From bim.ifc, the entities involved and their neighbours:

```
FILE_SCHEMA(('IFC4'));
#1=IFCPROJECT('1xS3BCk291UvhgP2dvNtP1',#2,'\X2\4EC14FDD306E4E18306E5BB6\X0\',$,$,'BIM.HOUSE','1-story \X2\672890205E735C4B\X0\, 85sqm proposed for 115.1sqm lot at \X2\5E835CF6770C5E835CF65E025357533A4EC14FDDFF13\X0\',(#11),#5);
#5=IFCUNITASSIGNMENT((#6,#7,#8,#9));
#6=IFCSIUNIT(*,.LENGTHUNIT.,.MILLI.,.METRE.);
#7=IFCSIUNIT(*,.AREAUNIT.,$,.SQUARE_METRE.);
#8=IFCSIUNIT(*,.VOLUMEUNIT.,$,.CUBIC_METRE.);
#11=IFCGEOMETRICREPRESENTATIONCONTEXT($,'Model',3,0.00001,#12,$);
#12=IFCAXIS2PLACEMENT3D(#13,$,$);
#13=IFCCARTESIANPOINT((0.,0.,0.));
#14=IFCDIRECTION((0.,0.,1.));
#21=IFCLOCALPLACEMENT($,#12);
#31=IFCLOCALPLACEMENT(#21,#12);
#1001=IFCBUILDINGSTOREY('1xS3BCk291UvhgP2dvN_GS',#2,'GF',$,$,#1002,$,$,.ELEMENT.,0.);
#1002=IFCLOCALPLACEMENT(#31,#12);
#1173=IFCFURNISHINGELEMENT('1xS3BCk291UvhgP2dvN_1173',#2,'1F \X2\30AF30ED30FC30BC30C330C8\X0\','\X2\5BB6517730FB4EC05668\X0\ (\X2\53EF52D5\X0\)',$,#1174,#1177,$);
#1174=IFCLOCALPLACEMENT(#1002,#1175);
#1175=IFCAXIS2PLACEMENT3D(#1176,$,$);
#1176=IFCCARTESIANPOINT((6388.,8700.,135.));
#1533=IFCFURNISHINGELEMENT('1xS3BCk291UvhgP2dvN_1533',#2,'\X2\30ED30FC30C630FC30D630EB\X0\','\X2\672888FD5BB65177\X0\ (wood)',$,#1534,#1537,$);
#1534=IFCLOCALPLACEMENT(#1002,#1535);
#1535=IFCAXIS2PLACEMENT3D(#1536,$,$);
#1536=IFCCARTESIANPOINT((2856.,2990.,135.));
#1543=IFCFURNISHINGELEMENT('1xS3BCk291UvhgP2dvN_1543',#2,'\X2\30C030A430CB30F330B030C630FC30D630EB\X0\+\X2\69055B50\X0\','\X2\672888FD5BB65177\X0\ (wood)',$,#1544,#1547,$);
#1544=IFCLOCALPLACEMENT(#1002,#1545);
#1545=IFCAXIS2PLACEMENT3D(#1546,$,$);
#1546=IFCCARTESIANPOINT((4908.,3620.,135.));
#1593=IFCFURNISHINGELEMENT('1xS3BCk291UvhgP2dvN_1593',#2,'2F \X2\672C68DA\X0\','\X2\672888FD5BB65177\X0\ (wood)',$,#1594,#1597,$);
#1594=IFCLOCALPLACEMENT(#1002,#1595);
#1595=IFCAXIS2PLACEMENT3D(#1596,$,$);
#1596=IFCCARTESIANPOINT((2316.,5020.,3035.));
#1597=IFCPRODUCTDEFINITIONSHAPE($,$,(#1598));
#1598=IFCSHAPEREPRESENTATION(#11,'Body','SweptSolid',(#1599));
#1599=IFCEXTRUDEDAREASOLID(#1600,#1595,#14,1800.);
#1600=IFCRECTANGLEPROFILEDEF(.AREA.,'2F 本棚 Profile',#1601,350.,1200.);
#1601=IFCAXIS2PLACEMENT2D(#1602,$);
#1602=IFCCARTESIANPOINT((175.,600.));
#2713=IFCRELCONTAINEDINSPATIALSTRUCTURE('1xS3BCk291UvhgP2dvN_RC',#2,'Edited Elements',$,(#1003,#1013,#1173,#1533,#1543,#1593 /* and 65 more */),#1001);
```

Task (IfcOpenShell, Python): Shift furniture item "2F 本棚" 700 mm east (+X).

```python
import ifcopenshell
import ifcopenshell.api.geometry
import ifcopenshell.util.placement
import ifcopenshell.util.unit

model = ifcopenshell.open("bim.ifc")
unit_scale = ifcopenshell.util.unit.calculate_unit_scale(model)

item = model.by_guid("1xS3BCk291UvhgP2dvN_1593")
matrix = ifcopenshell.util.placement.get_local_placement(item.ObjectPlacement)
matrix[0, 3] += 0.7 / unit_scale
ifcopenshell.api.geometry.edit_object_placement(model, product=item, matrix=matrix, is_si=False)

print(ifcopenshell.util.placement.get_local_placement(item.ObjectPlacement).round(3) + 0.0)

model.write("bim_edited.ifc")
```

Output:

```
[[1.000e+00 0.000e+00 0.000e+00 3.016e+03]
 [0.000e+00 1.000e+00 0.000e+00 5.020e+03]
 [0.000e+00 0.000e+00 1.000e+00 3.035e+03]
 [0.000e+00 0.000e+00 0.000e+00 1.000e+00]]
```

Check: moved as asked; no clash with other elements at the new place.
